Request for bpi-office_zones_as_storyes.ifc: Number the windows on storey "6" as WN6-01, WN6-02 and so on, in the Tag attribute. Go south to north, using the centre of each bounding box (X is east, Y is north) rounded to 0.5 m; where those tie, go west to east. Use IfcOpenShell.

First a look at what the model holds.

```python
import ifcopenshell
import ifcopenshell.util.element
import ifcopenshell.util.placement

model = ifcopenshell.open("bpi-office_zones_as_storyes.ifc")
print(model.schema)
storey = next(s for s in model.by_type("IfcBuildingStorey") if s.Name == "6")
windows = [e for e in ifcopenshell.util.element.get_decomposition(storey) if e.is_a("IfcWindow")]
for e in sorted(windows, key=lambda e: e.id()):
    origin = ifcopenshell.util.placement.get_local_placement(e.ObjectPlacement)[:3, 3]
    print(e.id(), e.Tag, e.Name, origin.round(2) + 0.0, sep=" | ")
```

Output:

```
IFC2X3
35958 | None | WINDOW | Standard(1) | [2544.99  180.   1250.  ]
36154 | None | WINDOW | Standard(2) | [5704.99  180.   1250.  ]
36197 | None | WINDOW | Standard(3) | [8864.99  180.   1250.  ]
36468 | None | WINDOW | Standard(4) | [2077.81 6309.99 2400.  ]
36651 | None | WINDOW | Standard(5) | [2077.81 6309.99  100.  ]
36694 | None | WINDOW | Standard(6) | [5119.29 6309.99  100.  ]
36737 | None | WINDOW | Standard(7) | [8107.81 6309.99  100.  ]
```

```python
import ifcopenshell
import ifcopenshell.geom
import ifcopenshell.util.element
import ifcopenshell.util.shape

model = ifcopenshell.open("bpi-office_zones_as_storyes.ifc")
settings = ifcopenshell.geom.settings()
settings.set("use-world-coords", True)


def centre(element):
    shape = ifcopenshell.geom.create_shape(settings, element)
    return ifcopenshell.util.shape.get_bbox_centroid(shape.geometry)


storey = next(s for s in model.by_type("IfcBuildingStorey") if s.Name == "6")
windows = [e for e in ifcopenshell.util.element.get_decomposition(storey) if e.is_a("IfcWindow")]

# Insertion points can sit at a corner or the storey origin, so sort by the geometry (in metres).
centres = {e: centre(e) for e in windows}
windows.sort(key=lambda e: (round(centres[e][1] / 0.5), centres[e][0]))

for i, e in enumerate(windows, start=1):
    number = f"WN6-{i:02d}"
    e.Tag = number
    print(e.id(), number)

model.write("bpi-office_zones_as_storyes-out.ifc")
```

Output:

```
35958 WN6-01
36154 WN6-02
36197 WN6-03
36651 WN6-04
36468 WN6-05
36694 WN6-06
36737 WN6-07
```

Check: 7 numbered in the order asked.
